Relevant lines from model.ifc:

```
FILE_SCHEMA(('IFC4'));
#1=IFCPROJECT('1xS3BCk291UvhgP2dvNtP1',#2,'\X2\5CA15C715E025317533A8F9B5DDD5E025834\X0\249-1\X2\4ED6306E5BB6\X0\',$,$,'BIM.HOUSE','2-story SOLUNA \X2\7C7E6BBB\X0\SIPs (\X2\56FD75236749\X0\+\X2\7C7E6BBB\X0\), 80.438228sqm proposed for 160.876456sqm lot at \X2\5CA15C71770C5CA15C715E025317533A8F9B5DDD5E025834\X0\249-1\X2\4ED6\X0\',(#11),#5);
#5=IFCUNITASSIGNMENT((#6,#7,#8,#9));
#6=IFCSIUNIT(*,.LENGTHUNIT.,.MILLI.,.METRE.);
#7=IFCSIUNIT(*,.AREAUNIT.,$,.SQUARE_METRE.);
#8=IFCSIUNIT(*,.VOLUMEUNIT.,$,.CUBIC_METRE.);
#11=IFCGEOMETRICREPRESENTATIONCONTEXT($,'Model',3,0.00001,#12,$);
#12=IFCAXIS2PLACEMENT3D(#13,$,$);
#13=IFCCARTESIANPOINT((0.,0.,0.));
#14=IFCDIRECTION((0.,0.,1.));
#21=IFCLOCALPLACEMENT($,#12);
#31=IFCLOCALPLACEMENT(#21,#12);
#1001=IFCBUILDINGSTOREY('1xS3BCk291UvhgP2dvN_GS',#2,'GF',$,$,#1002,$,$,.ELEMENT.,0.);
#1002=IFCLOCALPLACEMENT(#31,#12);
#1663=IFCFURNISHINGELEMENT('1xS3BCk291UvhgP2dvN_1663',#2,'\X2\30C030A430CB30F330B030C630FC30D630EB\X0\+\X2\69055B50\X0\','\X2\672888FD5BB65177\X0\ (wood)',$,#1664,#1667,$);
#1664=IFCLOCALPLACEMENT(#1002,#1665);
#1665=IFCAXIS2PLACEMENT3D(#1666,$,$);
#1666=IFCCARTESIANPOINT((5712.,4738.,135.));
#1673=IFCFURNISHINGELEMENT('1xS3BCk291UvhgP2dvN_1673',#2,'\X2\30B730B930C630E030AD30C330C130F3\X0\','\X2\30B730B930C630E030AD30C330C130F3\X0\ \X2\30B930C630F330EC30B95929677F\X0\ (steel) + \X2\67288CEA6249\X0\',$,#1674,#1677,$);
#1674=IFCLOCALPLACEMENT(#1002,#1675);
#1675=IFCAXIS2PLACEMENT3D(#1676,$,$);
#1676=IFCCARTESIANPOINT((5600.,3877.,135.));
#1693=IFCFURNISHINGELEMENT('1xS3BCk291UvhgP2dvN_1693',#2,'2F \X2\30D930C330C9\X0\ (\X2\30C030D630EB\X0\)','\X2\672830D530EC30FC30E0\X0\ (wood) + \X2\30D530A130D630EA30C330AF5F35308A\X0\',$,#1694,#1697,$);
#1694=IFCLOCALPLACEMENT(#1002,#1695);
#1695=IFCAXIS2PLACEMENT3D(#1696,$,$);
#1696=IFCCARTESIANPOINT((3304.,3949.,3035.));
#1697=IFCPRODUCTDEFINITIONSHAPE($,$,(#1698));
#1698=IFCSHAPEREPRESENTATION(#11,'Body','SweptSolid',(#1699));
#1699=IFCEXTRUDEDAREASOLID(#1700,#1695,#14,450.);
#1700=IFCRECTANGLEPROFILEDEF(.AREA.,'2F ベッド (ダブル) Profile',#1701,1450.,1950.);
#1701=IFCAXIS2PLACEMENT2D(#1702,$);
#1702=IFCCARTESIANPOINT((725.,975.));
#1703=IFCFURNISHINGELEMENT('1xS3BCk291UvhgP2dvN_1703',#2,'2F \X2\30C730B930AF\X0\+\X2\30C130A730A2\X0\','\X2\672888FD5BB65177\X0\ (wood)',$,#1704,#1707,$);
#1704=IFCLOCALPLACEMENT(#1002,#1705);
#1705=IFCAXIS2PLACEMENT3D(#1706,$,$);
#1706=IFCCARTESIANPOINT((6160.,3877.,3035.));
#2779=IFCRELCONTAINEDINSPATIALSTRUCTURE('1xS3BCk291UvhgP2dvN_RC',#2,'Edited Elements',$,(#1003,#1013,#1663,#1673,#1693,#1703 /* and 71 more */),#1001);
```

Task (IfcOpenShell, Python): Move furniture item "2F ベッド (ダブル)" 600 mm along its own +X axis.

```python
import ifcopenshell
import ifcopenshell.api.geometry
import ifcopenshell.util.placement
import ifcopenshell.util.unit

model = ifcopenshell.open("model.ifc")
unit_scale = ifcopenshell.util.unit.calculate_unit_scale(model)

item = model.by_guid("1xS3BCk291UvhgP2dvN_1693")
matrix = ifcopenshell.util.placement.get_local_placement(item.ObjectPlacement)
matrix[:3, 3] += matrix[:3, 0] * 0.6 / unit_scale
ifcopenshell.api.geometry.edit_object_placement(model, product=item, matrix=matrix, is_si=False)

print(ifcopenshell.util.placement.get_local_placement(item.ObjectPlacement).round(3) + 0.0)

model.write("model-out.ifc")
```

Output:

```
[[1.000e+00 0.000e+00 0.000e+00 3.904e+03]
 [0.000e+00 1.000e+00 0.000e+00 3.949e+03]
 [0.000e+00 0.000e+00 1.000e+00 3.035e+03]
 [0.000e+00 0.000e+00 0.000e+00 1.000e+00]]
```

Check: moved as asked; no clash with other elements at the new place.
